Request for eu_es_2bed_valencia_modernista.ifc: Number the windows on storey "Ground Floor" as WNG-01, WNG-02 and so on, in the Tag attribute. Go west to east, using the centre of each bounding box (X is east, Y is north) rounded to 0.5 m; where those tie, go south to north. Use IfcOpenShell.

First a look at what the model holds.

```python
import ifcopenshell
import ifcopenshell.util.element
import ifcopenshell.util.placement

model = ifcopenshell.open("eu_es_2bed_valencia_modernista.ifc")
print(model.schema)
storey = next(s for s in model.by_type("IfcBuildingStorey") if s.Name == "Ground Floor")
windows = [e for e in ifcopenshell.util.element.get_decomposition(storey) if e.is_a("IfcWindow")]
for e in sorted(windows, key=lambda e: e.id()):
    origin = ifcopenshell.util.placement.get_local_placement(e.ObjectPlacement)[:3, 3]
    print(e.id(), e.Tag, e.Name, origin.round(2) + 0.0, sep=" | ")
```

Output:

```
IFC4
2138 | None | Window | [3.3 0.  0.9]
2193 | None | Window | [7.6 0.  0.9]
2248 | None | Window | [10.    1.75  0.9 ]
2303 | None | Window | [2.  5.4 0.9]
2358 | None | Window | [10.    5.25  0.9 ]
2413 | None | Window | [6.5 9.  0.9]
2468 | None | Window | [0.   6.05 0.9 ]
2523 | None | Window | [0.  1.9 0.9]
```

```python
import ifcopenshell
import ifcopenshell.geom
import ifcopenshell.util.element
import ifcopenshell.util.shape

model = ifcopenshell.open("eu_es_2bed_valencia_modernista.ifc")
settings = ifcopenshell.geom.settings()
settings.set("use-world-coords", True)


def centre(element):
    shape = ifcopenshell.geom.create_shape(settings, element)
    return ifcopenshell.util.shape.get_bbox_centroid(shape.geometry)


storey = next(s for s in model.by_type("IfcBuildingStorey") if s.Name == "Ground Floor")
windows = [e for e in ifcopenshell.util.element.get_decomposition(storey) if e.is_a("IfcWindow")]

# Insertion points can sit at a corner or the storey origin, so sort by the geometry (in metres).
centres = {e: centre(e) for e in windows}
windows.sort(key=lambda e: (round(centres[e][0] / 0.5), centres[e][1]))

for i, e in enumerate(windows, start=1):
    number = f"WNG-{i:02d}"
    e.Tag = number
    print(e.id(), number)

model.write("eu_es_2bed_valencia_modernista_rev.ifc")
```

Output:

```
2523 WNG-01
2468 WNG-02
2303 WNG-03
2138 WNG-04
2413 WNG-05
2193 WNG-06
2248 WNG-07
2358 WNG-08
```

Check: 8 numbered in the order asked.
